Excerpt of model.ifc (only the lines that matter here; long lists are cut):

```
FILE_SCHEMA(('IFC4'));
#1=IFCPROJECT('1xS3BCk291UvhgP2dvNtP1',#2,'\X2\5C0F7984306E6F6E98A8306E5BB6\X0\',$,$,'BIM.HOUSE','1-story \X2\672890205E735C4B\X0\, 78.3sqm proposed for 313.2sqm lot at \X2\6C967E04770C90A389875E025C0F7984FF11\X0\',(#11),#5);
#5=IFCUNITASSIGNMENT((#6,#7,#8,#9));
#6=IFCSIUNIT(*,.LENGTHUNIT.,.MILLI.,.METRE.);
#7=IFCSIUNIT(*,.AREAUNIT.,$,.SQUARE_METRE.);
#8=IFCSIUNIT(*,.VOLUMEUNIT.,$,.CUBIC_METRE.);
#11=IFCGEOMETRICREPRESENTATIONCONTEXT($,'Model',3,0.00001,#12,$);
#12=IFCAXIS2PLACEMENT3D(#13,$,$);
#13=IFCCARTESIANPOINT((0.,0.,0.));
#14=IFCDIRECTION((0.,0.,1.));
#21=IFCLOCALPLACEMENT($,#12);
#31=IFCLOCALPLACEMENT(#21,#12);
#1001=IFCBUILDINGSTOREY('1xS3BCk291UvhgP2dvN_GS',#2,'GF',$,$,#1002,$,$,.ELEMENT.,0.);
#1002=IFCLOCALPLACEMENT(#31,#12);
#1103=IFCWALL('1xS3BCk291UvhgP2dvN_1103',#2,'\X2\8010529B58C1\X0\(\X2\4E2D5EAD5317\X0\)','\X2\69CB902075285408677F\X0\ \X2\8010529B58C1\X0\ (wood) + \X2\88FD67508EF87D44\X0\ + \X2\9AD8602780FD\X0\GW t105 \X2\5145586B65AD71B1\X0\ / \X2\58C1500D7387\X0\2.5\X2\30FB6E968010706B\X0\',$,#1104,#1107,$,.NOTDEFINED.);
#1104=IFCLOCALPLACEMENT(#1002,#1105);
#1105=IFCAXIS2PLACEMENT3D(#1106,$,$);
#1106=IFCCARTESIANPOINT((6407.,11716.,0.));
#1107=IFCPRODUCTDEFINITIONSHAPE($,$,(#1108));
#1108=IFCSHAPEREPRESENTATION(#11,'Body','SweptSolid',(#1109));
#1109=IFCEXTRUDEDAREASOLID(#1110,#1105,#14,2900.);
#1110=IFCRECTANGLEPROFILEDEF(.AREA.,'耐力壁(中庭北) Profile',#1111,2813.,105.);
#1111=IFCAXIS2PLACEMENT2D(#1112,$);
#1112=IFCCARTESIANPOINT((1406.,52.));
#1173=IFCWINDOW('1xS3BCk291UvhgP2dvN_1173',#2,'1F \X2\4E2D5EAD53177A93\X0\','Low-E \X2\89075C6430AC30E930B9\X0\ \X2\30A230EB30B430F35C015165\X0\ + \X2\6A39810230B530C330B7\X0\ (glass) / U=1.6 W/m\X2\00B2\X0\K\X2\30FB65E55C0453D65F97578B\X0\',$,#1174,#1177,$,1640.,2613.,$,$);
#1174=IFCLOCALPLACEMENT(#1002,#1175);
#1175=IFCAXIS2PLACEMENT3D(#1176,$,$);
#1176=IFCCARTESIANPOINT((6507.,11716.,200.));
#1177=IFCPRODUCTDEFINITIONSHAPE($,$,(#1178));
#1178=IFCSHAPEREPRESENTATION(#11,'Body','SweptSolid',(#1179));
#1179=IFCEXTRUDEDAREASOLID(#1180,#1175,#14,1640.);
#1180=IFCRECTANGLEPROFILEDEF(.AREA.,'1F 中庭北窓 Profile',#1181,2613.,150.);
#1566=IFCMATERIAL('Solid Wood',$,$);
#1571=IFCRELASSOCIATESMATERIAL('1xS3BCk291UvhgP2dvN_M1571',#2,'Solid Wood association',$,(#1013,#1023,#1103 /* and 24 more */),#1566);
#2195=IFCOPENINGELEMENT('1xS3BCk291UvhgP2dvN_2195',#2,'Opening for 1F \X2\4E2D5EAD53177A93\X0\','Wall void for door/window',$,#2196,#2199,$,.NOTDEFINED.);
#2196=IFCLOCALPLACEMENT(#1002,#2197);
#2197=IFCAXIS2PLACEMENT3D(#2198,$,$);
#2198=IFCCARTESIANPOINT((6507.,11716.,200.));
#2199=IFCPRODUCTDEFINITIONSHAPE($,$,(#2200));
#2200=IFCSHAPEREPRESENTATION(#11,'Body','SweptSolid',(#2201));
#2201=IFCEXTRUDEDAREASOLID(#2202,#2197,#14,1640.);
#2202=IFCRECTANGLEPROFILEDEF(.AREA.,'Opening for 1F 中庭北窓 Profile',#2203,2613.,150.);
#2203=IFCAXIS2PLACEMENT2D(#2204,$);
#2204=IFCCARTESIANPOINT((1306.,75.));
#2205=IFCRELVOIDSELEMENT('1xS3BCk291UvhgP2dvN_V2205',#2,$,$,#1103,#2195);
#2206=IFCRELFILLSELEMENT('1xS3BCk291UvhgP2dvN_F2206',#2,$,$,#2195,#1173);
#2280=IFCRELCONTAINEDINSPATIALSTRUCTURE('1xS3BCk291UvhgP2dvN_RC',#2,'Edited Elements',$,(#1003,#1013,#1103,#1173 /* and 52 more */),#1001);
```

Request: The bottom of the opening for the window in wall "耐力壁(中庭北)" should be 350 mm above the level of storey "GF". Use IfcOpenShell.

```python
import numpy as np
import ifcopenshell
import ifcopenshell.api.geometry
import ifcopenshell.geom
import ifcopenshell.util.element
import ifcopenshell.util.placement
import ifcopenshell.util.shape
import ifcopenshell.util.unit

model = ifcopenshell.open("model.ifc")
unit_scale = ifcopenshell.util.unit.calculate_unit_scale(model)

window = model.by_guid("1xS3BCk291UvhgP2dvN_1173")
opening = window.FillsVoids[0].RelatingOpeningElement
storey = ifcopenshell.util.element.get_container(window, ifc_class="IfcBuildingStorey")
level = ifcopenshell.util.placement.get_local_placement(storey.ObjectPlacement)[2, 3]

# The opening's origin need not be at the sill, so measure its lowest point.
shape = ifcopenshell.geom.create_shape(ifcopenshell.geom.settings(), opening)
bottom = ifcopenshell.util.shape.get_shape_bottom_elevation(shape, shape.geometry) / unit_scale
dz = level + 0.35 / unit_scale - bottom

shift = np.array([0.0, 0.0, dz])
# The window is not placed relative to its opening, so move both.
for product in (opening, window):
    matrix = ifcopenshell.util.placement.get_local_placement(product.ObjectPlacement)
    matrix[:3, 3] += shift
    ifcopenshell.api.geometry.edit_object_placement(model, product=product, matrix=matrix, is_si=False)

print(f"moved by {dz * unit_scale:+.3f} m")

model.write("model_updated.ifc")
```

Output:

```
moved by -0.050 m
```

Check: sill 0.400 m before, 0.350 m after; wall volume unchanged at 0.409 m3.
